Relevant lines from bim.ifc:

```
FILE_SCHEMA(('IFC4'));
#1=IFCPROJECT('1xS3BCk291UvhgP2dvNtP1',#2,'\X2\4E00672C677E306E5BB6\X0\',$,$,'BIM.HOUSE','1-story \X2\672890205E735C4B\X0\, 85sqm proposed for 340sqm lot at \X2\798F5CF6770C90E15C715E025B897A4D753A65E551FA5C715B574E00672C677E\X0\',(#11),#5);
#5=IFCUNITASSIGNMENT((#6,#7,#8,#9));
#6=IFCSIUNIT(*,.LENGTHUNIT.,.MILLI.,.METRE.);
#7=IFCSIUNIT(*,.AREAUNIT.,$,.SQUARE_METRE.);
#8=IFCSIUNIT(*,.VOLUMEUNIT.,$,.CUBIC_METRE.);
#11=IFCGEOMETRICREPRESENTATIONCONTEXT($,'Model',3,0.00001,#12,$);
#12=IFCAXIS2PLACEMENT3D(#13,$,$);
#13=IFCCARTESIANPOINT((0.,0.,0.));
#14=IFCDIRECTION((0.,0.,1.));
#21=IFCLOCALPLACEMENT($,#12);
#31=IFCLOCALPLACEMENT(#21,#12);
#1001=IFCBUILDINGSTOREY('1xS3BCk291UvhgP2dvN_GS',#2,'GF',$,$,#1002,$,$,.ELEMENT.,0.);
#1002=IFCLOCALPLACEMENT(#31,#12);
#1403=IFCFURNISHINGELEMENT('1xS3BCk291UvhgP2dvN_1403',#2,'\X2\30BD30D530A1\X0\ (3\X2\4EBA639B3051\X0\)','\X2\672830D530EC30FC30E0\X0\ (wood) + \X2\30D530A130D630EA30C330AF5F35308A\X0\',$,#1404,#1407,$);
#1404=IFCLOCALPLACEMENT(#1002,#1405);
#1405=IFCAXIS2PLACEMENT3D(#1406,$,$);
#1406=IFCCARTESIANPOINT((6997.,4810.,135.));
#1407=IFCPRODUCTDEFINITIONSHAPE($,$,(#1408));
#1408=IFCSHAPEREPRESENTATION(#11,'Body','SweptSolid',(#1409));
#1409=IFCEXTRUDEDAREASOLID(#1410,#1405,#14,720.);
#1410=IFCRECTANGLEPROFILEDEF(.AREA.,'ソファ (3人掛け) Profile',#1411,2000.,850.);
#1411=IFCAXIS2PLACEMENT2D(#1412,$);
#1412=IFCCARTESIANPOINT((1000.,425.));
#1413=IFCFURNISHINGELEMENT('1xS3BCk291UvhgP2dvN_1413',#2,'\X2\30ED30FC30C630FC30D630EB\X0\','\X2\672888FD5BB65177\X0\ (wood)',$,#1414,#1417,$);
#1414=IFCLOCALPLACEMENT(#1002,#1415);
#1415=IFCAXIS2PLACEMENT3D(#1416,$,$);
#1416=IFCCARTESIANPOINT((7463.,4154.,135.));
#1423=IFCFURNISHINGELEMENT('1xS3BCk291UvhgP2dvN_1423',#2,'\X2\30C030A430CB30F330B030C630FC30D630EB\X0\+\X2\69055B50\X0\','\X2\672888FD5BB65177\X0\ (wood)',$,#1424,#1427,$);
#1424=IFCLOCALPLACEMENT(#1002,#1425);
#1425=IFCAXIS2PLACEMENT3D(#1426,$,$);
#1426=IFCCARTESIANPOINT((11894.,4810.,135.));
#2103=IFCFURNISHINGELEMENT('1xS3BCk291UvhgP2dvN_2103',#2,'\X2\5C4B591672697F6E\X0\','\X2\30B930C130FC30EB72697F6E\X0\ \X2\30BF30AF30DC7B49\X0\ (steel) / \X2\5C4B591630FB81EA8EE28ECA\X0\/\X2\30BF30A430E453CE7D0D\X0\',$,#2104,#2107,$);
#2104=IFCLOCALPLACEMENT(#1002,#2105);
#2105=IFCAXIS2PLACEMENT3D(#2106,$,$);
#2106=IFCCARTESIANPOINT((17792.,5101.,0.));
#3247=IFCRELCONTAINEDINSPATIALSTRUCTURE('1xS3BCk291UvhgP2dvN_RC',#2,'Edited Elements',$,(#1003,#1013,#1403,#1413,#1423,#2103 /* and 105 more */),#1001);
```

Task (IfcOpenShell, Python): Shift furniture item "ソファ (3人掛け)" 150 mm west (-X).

```python
import ifcopenshell
import ifcopenshell.api.geometry
import ifcopenshell.util.placement
import ifcopenshell.util.unit

model = ifcopenshell.open("bim.ifc")
unit_scale = ifcopenshell.util.unit.calculate_unit_scale(model)

item = model.by_guid("1xS3BCk291UvhgP2dvN_1403")
matrix = ifcopenshell.util.placement.get_local_placement(item.ObjectPlacement)
matrix[0, 3] -= 0.15 / unit_scale
ifcopenshell.api.geometry.edit_object_placement(model, product=item, matrix=matrix, is_si=False)

print(ifcopenshell.util.placement.get_local_placement(item.ObjectPlacement).round(3) + 0.0)

model.write("bim_updated.ifc")
```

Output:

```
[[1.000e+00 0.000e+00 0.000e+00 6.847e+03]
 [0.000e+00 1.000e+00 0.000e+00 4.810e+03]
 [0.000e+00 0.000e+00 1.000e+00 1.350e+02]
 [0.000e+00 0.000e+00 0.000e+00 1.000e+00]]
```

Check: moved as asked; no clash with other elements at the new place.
